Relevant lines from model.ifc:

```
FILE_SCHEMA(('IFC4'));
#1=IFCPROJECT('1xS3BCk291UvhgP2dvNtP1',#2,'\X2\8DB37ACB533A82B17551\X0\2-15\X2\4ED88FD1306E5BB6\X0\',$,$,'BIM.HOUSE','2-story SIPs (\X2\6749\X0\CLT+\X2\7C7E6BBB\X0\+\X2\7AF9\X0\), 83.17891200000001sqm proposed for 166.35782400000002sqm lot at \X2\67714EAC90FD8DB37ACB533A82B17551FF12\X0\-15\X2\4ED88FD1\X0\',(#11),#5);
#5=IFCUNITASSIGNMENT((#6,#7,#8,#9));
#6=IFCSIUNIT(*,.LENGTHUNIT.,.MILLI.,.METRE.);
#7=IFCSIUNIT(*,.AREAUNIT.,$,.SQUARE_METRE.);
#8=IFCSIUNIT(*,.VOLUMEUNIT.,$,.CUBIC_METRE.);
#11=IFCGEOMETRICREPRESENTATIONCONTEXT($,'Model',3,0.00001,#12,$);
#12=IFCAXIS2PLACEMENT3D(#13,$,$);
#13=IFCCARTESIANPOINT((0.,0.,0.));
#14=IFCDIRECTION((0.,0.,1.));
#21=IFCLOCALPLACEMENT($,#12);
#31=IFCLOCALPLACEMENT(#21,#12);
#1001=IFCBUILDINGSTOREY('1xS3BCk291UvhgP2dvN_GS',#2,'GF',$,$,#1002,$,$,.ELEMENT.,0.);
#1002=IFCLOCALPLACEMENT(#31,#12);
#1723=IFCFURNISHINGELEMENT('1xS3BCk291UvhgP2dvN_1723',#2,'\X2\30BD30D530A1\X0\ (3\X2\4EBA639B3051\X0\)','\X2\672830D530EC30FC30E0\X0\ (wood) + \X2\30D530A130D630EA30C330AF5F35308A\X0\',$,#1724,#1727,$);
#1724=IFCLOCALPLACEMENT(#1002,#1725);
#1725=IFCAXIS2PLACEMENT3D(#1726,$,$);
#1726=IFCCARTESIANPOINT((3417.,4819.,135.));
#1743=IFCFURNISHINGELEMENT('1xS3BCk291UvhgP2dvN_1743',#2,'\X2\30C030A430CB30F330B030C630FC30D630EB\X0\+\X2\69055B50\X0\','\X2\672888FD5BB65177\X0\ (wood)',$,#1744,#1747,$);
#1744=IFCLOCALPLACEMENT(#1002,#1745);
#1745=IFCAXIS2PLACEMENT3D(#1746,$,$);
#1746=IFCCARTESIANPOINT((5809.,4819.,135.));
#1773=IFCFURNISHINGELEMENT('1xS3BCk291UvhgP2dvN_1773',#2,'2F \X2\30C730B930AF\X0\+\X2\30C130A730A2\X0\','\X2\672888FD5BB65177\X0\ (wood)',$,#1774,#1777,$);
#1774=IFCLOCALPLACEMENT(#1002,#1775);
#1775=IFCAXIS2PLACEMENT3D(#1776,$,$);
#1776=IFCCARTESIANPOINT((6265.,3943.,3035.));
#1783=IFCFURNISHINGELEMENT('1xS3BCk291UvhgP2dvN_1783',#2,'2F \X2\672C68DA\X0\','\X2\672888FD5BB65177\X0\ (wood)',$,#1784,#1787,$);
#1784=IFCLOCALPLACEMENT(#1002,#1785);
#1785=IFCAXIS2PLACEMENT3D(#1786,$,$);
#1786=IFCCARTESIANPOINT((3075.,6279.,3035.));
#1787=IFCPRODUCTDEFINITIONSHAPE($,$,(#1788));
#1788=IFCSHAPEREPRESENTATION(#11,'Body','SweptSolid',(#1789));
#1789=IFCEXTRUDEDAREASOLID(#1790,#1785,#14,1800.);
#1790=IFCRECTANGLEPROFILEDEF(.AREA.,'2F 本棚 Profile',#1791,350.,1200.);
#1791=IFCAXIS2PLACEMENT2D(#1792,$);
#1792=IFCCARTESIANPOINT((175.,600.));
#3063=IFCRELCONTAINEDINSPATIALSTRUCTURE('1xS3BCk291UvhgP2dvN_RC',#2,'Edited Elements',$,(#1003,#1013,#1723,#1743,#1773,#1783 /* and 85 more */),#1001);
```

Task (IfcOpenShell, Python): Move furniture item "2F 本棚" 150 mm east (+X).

```python
import ifcopenshell
import ifcopenshell.api.geometry
import ifcopenshell.util.placement

model = ifcopenshell.open("model.ifc")

item = model.by_id(1783)
matrix = ifcopenshell.util.placement.get_local_placement(item.ObjectPlacement)
matrix[0, 3] += 150.0
ifcopenshell.api.geometry.edit_object_placement(model, product=item, matrix=matrix, is_si=False)

print(ifcopenshell.util.placement.get_local_placement(item.ObjectPlacement).round(3) + 0.0)

model.write("model-out.ifc")
```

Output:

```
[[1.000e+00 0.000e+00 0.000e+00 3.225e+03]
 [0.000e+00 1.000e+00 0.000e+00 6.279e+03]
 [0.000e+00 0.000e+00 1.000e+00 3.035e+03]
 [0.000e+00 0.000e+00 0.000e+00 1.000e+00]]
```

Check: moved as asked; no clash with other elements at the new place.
